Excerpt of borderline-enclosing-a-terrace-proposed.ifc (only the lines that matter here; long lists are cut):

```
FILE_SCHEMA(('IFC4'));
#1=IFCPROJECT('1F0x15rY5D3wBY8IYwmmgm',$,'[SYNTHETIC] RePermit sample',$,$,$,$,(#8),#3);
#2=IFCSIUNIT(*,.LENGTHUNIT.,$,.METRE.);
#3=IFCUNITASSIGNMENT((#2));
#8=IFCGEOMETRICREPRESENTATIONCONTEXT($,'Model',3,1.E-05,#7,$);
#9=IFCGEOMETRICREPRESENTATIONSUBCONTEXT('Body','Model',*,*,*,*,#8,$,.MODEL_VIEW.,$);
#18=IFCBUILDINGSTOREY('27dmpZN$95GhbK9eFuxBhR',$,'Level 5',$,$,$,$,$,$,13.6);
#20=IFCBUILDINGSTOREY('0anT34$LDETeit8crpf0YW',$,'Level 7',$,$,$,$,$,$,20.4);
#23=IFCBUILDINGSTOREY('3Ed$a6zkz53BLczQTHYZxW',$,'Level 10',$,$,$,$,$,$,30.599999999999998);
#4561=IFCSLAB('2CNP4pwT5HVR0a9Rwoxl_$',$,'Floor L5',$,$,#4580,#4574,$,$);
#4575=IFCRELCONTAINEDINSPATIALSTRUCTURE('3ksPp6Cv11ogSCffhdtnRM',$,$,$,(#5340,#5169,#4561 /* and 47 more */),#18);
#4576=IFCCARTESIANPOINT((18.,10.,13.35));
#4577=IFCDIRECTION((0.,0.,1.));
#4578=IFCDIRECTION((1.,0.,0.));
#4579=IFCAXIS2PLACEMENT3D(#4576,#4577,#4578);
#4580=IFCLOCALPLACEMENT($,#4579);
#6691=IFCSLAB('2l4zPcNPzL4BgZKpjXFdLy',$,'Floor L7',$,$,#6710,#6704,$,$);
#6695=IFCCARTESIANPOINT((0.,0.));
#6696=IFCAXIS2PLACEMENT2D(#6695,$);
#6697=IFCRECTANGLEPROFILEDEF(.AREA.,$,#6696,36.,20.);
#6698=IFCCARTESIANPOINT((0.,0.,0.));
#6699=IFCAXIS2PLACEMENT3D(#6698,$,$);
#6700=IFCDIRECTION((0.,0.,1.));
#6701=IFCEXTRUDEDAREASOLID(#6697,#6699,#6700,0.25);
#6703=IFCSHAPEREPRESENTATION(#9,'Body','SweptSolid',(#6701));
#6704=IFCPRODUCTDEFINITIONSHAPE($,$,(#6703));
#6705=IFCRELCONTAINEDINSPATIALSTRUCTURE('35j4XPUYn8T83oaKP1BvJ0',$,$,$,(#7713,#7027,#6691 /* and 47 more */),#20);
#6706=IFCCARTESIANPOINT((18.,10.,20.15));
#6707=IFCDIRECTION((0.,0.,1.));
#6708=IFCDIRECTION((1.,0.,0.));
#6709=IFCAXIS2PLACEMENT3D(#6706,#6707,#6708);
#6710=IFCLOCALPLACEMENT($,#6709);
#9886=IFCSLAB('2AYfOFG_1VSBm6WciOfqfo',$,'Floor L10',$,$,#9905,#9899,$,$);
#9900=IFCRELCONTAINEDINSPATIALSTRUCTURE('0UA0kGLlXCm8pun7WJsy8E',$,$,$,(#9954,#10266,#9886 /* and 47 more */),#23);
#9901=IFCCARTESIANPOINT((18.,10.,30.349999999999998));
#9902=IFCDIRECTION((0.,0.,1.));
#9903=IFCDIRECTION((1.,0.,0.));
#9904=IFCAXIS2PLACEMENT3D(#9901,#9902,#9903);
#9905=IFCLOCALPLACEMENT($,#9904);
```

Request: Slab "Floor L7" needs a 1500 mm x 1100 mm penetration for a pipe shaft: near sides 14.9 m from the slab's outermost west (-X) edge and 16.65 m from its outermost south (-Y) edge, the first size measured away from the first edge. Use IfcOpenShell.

```python
import numpy as np
import ifcopenshell
import ifcopenshell.api.feature
import ifcopenshell.api.geometry
import ifcopenshell.api.root
import ifcopenshell.geom
import ifcopenshell.util.placement
import ifcopenshell.util.representation
import ifcopenshell.util.shape
import ifcopenshell.util.unit

model = ifcopenshell.open("borderline-enclosing-a-terrace-proposed.ifc")
unit_scale = ifcopenshell.util.unit.calculate_unit_scale(model)
settings = ifcopenshell.geom.settings()


def volume(element):
    """Net volume in cubic metres, openings subtracted."""
    shape = ifcopenshell.geom.create_shape(settings, element)
    return ifcopenshell.util.shape.get_volume(shape.geometry)


slab = model.by_guid("2l4zPcNPzL4BgZKpjXFdLy")
before = volume(slab)

# Extent in the slab's own axes, in metres. The edges named are its -X and -Y sides.
slab_shape = ifcopenshell.geom.create_shape(settings, slab)
vertices = ifcopenshell.util.shape.get_vertices(slab_shape.geometry)
x_min, y_min, bottom = vertices.min(axis=0)
top = vertices[:, 2].max()

opening = ifcopenshell.api.root.create_entity(model, ifc_class="IfcOpeningElement", name="Pipe shaft opening", predefined_type="OPENING")
context = ifcopenshell.util.representation.get_context(model, "Model", "Body", "MODEL_VIEW")
width, depth = 1.5, 1.1
outline = [(0.0, 0.0), (width, 0.0), (width, depth), (0.0, depth), (0.0, 0.0)]
# Overshoot both faces by 50 mm so the cut is clean.
shape = ifcopenshell.api.geometry.add_slab_representation(
    model, context=context, depth=top - bottom + 0.1, polyline=outline
)
ifcopenshell.api.geometry.assign_representation(model, product=opening, representation=shape)

matrix = ifcopenshell.util.placement.get_local_placement(slab.ObjectPlacement)
matrix[:, 3] = matrix @ np.append(np.array([x_min + 14.9, y_min + 16.65, bottom - 0.05]) / unit_scale, 1.0)
ifcopenshell.api.geometry.edit_object_placement(model, product=opening, matrix=matrix, is_si=False)
ifcopenshell.api.feature.add_feature(model, feature=opening, element=slab)

after = volume(slab)

print(f"slab volume {before:.3f} -> {after:.3f} m3")

model.write("borderline-enclosing-a-terrace-proposed-out.ifc")
```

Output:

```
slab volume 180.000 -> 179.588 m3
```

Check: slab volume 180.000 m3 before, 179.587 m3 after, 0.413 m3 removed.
